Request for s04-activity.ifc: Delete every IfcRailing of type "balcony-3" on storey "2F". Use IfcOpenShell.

First a look at what the model holds.

```python
import ifcopenshell
import ifcopenshell.util.element

model = ifcopenshell.open("s04-activity.ifc")
print(model.schema)
storey = next(s for s in model.by_type("IfcBuildingStorey") if s.Name == "2F")
railings = [e for e in ifcopenshell.util.element.get_decomposition(storey) if e.is_a("IfcRailing")]
seen = {}
for e in railings:
    element_type = ifcopenshell.util.element.get_type(e)
    name = element_type.Name if element_type not in (None, e) else None
    seen[name] = seen.get(name, 0) + 1
for name, count in sorted(seen.items(), key=str):
    print(count, "x", name)
```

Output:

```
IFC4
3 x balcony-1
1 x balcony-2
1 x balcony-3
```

```python
import ifcopenshell
import ifcopenshell.api.root
import ifcopenshell.util.element

model = ifcopenshell.open("s04-activity.ifc")

storey = next(s for s in model.by_type("IfcBuildingStorey") if s.Name == "2F")
railings = [e for e in ifcopenshell.util.element.get_decomposition(storey) if e.is_a("IfcRailing")]
targets = [e for e in railings if (t := ifcopenshell.util.element.get_type(e)) not in (None, e) and t.Name == "balcony-3"]

for e in targets:
    ifcopenshell.api.root.remove_product(model, product=e)
print(len(targets), "removed")

model.write("s04-activity-out.ifc")
```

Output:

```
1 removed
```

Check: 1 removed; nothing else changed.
